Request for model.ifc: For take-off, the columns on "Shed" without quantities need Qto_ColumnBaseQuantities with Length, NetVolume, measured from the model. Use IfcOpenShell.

First a look at what the model holds.

```python
import ifcopenshell
import ifcopenshell.util.element
import ifcopenshell.util.unit

model = ifcopenshell.open("model.ifc")
print(model.schema)
for unit_type in ("LENGTHUNIT", "AREAUNIT", "VOLUMEUNIT"):
    print(unit_type, ifcopenshell.util.unit.calculate_unit_scale(model, unit_type))
storey = next(s for s in model.by_type("IfcBuildingStorey") if s.Name == "Shed")
columns = [e for e in ifcopenshell.util.element.get_decomposition(storey) if e.is_a("IfcColumn")]
for e in sorted(columns, key=lambda e: e.id()):
    print(e.id(), e.is_a(), e.Name, list(ifcopenshell.util.element.get_psets(e, qtos_only=True)), sep=" | ")
```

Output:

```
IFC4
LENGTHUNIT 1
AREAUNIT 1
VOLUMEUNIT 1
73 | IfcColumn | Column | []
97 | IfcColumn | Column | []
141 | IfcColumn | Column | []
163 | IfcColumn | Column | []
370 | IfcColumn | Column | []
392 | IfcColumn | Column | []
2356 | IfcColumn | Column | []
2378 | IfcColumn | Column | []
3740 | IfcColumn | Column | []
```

```python
import ifcopenshell
import ifcopenshell.api.pset
import ifcopenshell.geom
import ifcopenshell.util.element
import ifcopenshell.util.shape
import ifcopenshell.util.unit

model = ifcopenshell.open("model.ifc")
unit_scale = ifcopenshell.util.unit.calculate_unit_scale(model)
volume_scale = ifcopenshell.util.unit.calculate_unit_scale(model, "VOLUMEUNIT")
settings = ifcopenshell.geom.settings()

storey = next(s for s in model.by_type("IfcBuildingStorey") if s.Name == "Shed")
columns = [e for e in ifcopenshell.util.element.get_decomposition(storey) if e.is_a("IfcColumn")]

for e in sorted(columns, key=lambda e: e.id()):
    if ifcopenshell.util.element.get_psets(e, qtos_only=True, should_inherit=False):
        continue
    # Geometry comes back in metres, in the element's own axes.
    shape = ifcopenshell.geom.create_shape(settings, e)
    values = {
        "Length": ifcopenshell.util.shape.get_z(shape.geometry) / unit_scale,
        "NetVolume": ifcopenshell.util.shape.get_volume(shape.geometry) / volume_scale,
    }
    qto = ifcopenshell.api.pset.add_qto(model, product=e, name="Qto_ColumnBaseQuantities")
    ifcopenshell.api.pset.edit_qto(model, qto=qto, properties=values)
    print(e.id(), {k: round(v, 3) for k, v in values.items()})

model.write("model_edited.ifc")
```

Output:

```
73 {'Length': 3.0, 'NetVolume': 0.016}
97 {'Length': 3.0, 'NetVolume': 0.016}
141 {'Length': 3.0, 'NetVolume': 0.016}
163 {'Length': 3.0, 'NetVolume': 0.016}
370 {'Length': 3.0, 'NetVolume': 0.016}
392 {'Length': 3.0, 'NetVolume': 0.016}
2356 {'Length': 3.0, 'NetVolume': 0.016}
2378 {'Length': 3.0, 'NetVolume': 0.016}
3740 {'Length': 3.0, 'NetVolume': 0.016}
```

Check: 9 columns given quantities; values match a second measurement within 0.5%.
